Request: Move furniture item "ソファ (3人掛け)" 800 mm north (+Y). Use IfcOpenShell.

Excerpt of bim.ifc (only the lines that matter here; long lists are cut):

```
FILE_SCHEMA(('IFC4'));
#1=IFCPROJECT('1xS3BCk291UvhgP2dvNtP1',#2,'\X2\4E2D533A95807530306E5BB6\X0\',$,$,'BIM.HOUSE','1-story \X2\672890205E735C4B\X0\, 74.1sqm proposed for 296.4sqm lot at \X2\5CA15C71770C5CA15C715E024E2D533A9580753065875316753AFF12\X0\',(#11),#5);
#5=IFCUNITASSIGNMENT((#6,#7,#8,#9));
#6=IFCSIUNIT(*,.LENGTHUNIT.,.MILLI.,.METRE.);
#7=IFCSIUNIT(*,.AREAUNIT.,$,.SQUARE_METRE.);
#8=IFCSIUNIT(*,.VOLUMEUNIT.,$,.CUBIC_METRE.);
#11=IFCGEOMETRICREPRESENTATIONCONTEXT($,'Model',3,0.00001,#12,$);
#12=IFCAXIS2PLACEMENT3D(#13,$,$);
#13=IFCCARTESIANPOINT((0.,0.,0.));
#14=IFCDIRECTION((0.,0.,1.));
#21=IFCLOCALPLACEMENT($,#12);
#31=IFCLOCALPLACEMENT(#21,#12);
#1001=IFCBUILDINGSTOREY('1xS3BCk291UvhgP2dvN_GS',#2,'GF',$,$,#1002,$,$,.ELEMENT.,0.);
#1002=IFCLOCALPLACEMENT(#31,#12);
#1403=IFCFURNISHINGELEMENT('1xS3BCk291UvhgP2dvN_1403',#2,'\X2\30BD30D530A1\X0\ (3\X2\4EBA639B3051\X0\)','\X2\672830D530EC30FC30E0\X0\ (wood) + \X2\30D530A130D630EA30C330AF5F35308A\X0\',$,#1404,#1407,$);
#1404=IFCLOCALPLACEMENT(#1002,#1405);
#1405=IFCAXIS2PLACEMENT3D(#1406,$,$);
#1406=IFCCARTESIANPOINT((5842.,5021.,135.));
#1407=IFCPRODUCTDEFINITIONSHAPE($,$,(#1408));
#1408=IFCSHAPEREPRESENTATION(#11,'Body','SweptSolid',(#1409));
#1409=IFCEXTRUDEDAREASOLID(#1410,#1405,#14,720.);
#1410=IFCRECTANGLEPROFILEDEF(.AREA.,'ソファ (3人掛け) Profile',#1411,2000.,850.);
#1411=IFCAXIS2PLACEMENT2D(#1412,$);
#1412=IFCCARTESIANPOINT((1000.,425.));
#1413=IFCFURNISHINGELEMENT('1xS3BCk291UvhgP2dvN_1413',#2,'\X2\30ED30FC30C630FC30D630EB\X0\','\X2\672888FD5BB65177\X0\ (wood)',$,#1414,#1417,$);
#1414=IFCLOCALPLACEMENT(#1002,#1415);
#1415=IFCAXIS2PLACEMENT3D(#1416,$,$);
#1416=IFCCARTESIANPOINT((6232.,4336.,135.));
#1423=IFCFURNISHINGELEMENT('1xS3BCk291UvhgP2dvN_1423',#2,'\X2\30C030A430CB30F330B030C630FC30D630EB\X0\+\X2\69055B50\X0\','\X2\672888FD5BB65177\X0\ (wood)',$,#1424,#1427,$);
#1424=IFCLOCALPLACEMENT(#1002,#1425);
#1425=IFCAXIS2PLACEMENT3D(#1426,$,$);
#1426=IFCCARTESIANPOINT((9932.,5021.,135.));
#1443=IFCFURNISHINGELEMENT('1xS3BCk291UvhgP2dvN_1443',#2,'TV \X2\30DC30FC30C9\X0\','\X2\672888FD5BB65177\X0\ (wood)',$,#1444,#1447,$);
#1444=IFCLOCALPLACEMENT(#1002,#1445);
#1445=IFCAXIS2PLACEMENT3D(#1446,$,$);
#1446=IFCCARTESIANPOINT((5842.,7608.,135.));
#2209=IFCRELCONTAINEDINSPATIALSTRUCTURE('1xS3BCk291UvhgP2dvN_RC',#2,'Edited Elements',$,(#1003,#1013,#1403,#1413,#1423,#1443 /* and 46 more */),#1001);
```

```python
import ifcopenshell
import ifcopenshell.api.geometry
import ifcopenshell.util.placement
import ifcopenshell.util.unit

model = ifcopenshell.open("bim.ifc")
unit_scale = ifcopenshell.util.unit.calculate_unit_scale(model)

item = model.by_guid("1xS3BCk291UvhgP2dvN_1403")
matrix = ifcopenshell.util.placement.get_local_placement(item.ObjectPlacement)
matrix[1, 3] += 0.8 / unit_scale
ifcopenshell.api.geometry.edit_object_placement(model, product=item, matrix=matrix, is_si=False)

print(ifcopenshell.util.placement.get_local_placement(item.ObjectPlacement).round(3) + 0.0)

model.write("bim_v2.ifc")
```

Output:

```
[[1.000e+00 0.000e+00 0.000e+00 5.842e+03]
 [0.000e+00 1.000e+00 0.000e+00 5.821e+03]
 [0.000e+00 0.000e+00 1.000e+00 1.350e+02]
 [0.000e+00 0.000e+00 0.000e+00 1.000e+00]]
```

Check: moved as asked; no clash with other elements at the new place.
